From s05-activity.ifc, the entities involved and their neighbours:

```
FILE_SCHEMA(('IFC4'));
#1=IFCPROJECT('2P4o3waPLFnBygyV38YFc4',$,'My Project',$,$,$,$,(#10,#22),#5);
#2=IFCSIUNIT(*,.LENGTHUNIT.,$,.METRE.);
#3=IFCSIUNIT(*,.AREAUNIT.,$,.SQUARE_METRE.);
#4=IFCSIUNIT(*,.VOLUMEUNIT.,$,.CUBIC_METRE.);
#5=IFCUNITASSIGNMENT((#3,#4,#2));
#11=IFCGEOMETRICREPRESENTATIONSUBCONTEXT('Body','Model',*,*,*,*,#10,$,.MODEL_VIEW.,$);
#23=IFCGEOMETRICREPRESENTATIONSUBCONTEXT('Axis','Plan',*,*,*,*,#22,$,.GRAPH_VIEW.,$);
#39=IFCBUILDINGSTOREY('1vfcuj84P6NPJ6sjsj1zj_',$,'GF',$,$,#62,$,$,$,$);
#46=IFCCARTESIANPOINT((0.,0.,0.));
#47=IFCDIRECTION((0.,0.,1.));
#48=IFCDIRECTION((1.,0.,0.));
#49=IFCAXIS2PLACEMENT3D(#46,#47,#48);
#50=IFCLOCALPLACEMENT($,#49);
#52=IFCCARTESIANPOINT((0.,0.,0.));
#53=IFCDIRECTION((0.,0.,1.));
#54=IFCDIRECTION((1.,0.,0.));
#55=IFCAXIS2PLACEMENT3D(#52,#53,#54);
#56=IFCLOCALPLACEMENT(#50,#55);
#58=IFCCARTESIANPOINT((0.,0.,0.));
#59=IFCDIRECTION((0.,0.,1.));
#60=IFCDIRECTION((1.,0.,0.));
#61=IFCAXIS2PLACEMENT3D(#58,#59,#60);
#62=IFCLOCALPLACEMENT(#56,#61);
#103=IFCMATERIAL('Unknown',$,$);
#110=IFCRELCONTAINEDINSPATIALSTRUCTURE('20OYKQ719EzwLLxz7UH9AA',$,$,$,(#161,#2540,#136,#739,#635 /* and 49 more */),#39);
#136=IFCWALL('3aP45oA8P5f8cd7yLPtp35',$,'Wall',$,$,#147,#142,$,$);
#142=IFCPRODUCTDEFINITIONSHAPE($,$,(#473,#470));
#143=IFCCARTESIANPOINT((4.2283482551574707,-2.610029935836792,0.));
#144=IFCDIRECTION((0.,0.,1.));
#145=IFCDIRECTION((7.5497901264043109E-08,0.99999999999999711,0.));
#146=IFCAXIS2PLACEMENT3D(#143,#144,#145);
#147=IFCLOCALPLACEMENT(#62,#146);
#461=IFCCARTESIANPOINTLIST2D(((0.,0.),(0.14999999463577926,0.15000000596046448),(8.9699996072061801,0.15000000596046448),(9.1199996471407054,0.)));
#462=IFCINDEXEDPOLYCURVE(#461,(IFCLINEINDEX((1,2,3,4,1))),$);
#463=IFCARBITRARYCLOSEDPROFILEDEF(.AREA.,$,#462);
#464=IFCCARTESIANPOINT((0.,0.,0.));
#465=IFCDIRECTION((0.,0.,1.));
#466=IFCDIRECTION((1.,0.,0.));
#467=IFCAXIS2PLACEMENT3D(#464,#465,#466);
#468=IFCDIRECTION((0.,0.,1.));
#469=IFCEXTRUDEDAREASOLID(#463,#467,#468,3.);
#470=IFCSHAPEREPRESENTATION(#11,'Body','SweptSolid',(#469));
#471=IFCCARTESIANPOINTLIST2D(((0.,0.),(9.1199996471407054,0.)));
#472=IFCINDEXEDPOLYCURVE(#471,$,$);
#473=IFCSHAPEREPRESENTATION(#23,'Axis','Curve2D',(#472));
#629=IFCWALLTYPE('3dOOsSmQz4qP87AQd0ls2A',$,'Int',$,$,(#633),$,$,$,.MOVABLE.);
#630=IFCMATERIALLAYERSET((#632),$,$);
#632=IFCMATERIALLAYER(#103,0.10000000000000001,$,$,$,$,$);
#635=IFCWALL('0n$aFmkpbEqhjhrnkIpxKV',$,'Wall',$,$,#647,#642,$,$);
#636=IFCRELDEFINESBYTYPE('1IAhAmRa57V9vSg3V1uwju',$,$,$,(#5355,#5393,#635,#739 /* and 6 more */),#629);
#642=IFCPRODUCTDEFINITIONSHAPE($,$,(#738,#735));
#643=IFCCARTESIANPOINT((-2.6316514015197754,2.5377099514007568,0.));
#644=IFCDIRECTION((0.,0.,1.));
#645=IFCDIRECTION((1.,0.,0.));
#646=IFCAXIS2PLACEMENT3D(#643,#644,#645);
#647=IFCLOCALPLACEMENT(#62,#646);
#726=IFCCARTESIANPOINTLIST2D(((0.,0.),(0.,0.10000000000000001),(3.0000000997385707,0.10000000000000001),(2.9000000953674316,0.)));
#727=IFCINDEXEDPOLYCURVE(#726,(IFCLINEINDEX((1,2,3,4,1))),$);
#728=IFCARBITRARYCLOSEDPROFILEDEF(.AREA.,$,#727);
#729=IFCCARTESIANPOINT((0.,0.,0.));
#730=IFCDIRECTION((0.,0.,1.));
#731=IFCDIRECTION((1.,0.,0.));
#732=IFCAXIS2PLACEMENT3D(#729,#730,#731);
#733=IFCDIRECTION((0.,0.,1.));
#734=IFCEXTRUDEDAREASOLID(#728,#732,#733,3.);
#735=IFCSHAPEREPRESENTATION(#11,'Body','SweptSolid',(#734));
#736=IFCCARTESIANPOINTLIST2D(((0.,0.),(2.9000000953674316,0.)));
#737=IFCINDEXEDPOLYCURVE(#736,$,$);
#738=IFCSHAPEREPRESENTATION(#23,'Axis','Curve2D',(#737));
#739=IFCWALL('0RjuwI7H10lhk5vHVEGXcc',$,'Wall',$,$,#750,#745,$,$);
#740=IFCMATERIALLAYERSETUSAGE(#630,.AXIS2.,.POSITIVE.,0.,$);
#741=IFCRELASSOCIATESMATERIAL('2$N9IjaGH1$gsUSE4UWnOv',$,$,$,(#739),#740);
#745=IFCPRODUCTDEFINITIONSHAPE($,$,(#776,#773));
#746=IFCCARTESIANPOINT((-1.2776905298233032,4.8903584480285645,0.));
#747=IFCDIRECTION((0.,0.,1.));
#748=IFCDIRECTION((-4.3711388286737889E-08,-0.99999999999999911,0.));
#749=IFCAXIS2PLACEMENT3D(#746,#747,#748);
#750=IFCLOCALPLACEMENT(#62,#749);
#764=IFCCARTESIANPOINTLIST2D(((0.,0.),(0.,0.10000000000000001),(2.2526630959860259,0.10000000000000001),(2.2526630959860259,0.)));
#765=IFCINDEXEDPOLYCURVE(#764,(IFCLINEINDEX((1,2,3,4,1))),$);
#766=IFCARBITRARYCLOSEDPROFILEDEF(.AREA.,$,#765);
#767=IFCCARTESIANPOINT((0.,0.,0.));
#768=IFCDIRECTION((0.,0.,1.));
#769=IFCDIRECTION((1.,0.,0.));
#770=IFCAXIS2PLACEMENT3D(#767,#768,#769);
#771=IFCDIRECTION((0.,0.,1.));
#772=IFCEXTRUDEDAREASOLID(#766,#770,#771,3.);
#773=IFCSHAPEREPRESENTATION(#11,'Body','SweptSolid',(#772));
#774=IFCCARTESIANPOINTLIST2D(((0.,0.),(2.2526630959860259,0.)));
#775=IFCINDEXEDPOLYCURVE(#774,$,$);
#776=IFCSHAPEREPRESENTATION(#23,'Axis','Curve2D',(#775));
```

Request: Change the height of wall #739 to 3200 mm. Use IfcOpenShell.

```python
import ifcopenshell
import ifcopenshell.geom
import ifcopenshell.util.representation
import ifcopenshell.util.shape

model = ifcopenshell.open("s05-activity.ifc")
settings = ifcopenshell.geom.settings()


def volume(element):
    """Net volume in cubic metres, openings subtracted."""
    shape = ifcopenshell.geom.create_shape(settings, element)
    return ifcopenshell.util.shape.get_volume(shape.geometry)


wall = model.by_id(739)
before = volume(wall)

body = ifcopenshell.util.representation.get_representation(wall, "Model", "Body")
solid = body.Items[0]
old_height = solid.Depth
solid.Depth = 3.2
after = volume(wall)

print(f"height {old_height:g} -> {solid.Depth:g}, volume {before:.3f} -> {after:.3f} m3")

model.write("s05-activity_updated.ifc")
```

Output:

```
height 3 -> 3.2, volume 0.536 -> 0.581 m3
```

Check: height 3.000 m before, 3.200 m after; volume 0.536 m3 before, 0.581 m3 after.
